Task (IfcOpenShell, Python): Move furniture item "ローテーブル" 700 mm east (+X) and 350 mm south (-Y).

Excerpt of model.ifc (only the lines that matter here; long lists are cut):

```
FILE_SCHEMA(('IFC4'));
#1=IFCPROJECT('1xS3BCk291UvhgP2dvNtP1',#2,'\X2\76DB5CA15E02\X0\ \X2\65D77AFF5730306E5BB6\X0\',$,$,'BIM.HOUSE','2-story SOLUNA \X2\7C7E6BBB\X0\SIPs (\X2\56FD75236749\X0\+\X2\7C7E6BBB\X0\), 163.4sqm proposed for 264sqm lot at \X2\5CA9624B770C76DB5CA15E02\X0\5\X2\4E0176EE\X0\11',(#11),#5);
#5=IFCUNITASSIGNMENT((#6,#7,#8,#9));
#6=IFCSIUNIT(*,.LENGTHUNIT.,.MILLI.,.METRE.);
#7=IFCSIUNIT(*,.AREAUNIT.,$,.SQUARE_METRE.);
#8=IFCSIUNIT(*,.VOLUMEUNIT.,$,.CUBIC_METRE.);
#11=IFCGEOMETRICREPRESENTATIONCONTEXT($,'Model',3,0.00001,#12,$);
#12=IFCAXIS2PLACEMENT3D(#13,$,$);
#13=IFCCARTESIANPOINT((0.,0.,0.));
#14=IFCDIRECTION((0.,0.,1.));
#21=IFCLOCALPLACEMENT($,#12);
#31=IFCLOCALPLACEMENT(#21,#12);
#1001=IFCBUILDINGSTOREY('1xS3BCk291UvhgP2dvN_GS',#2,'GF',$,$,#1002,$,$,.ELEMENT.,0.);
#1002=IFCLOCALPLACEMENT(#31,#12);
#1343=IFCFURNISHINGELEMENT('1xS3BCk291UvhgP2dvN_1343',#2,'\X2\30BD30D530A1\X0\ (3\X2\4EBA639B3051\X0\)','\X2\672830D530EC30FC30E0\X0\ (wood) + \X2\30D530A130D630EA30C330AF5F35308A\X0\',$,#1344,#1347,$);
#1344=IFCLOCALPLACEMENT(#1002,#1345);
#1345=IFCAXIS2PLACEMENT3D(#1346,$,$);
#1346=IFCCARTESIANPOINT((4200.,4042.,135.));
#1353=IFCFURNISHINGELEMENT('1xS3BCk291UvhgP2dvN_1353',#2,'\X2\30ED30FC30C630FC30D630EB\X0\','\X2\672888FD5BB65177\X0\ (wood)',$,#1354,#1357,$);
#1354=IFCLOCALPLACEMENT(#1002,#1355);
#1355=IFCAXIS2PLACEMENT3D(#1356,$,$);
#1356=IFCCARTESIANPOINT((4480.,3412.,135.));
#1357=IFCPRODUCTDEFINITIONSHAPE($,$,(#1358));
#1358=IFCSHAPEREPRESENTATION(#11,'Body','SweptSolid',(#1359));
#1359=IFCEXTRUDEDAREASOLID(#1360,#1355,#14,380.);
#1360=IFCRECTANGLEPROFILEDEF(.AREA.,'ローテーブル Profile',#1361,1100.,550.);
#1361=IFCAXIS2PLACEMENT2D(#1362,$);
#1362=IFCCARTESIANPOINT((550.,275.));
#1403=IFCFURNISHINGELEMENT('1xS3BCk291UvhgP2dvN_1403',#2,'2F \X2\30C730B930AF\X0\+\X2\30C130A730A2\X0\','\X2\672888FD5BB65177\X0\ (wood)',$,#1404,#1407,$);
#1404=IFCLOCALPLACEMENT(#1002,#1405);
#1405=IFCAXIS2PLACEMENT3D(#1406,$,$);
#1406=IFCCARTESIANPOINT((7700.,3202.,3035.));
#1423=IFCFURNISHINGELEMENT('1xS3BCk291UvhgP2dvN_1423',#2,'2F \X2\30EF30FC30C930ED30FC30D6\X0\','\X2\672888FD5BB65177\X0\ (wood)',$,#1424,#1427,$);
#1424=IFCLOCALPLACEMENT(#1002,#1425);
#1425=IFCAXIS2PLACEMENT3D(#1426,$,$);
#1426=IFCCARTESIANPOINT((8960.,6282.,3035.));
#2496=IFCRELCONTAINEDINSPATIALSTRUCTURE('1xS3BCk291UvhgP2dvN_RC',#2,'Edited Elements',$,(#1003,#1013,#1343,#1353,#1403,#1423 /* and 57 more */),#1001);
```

```python
import ifcopenshell
import ifcopenshell.api.geometry
import ifcopenshell.util.placement
import ifcopenshell.util.unit

model = ifcopenshell.open("model.ifc")
unit_scale = ifcopenshell.util.unit.calculate_unit_scale(model)

item = model.by_guid("1xS3BCk291UvhgP2dvN_1353")
matrix = ifcopenshell.util.placement.get_local_placement(item.ObjectPlacement)
matrix[0, 3] += 0.7 / unit_scale
matrix[1, 3] -= 0.35 / unit_scale
ifcopenshell.api.geometry.edit_object_placement(model, product=item, matrix=matrix, is_si=False)

print(ifcopenshell.util.placement.get_local_placement(item.ObjectPlacement).round(3) + 0.0)

model.write("model-out.ifc")
```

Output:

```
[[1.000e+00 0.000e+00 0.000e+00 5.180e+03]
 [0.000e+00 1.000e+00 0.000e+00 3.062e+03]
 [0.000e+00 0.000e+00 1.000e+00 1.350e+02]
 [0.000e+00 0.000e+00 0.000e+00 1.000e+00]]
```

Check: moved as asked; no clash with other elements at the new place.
